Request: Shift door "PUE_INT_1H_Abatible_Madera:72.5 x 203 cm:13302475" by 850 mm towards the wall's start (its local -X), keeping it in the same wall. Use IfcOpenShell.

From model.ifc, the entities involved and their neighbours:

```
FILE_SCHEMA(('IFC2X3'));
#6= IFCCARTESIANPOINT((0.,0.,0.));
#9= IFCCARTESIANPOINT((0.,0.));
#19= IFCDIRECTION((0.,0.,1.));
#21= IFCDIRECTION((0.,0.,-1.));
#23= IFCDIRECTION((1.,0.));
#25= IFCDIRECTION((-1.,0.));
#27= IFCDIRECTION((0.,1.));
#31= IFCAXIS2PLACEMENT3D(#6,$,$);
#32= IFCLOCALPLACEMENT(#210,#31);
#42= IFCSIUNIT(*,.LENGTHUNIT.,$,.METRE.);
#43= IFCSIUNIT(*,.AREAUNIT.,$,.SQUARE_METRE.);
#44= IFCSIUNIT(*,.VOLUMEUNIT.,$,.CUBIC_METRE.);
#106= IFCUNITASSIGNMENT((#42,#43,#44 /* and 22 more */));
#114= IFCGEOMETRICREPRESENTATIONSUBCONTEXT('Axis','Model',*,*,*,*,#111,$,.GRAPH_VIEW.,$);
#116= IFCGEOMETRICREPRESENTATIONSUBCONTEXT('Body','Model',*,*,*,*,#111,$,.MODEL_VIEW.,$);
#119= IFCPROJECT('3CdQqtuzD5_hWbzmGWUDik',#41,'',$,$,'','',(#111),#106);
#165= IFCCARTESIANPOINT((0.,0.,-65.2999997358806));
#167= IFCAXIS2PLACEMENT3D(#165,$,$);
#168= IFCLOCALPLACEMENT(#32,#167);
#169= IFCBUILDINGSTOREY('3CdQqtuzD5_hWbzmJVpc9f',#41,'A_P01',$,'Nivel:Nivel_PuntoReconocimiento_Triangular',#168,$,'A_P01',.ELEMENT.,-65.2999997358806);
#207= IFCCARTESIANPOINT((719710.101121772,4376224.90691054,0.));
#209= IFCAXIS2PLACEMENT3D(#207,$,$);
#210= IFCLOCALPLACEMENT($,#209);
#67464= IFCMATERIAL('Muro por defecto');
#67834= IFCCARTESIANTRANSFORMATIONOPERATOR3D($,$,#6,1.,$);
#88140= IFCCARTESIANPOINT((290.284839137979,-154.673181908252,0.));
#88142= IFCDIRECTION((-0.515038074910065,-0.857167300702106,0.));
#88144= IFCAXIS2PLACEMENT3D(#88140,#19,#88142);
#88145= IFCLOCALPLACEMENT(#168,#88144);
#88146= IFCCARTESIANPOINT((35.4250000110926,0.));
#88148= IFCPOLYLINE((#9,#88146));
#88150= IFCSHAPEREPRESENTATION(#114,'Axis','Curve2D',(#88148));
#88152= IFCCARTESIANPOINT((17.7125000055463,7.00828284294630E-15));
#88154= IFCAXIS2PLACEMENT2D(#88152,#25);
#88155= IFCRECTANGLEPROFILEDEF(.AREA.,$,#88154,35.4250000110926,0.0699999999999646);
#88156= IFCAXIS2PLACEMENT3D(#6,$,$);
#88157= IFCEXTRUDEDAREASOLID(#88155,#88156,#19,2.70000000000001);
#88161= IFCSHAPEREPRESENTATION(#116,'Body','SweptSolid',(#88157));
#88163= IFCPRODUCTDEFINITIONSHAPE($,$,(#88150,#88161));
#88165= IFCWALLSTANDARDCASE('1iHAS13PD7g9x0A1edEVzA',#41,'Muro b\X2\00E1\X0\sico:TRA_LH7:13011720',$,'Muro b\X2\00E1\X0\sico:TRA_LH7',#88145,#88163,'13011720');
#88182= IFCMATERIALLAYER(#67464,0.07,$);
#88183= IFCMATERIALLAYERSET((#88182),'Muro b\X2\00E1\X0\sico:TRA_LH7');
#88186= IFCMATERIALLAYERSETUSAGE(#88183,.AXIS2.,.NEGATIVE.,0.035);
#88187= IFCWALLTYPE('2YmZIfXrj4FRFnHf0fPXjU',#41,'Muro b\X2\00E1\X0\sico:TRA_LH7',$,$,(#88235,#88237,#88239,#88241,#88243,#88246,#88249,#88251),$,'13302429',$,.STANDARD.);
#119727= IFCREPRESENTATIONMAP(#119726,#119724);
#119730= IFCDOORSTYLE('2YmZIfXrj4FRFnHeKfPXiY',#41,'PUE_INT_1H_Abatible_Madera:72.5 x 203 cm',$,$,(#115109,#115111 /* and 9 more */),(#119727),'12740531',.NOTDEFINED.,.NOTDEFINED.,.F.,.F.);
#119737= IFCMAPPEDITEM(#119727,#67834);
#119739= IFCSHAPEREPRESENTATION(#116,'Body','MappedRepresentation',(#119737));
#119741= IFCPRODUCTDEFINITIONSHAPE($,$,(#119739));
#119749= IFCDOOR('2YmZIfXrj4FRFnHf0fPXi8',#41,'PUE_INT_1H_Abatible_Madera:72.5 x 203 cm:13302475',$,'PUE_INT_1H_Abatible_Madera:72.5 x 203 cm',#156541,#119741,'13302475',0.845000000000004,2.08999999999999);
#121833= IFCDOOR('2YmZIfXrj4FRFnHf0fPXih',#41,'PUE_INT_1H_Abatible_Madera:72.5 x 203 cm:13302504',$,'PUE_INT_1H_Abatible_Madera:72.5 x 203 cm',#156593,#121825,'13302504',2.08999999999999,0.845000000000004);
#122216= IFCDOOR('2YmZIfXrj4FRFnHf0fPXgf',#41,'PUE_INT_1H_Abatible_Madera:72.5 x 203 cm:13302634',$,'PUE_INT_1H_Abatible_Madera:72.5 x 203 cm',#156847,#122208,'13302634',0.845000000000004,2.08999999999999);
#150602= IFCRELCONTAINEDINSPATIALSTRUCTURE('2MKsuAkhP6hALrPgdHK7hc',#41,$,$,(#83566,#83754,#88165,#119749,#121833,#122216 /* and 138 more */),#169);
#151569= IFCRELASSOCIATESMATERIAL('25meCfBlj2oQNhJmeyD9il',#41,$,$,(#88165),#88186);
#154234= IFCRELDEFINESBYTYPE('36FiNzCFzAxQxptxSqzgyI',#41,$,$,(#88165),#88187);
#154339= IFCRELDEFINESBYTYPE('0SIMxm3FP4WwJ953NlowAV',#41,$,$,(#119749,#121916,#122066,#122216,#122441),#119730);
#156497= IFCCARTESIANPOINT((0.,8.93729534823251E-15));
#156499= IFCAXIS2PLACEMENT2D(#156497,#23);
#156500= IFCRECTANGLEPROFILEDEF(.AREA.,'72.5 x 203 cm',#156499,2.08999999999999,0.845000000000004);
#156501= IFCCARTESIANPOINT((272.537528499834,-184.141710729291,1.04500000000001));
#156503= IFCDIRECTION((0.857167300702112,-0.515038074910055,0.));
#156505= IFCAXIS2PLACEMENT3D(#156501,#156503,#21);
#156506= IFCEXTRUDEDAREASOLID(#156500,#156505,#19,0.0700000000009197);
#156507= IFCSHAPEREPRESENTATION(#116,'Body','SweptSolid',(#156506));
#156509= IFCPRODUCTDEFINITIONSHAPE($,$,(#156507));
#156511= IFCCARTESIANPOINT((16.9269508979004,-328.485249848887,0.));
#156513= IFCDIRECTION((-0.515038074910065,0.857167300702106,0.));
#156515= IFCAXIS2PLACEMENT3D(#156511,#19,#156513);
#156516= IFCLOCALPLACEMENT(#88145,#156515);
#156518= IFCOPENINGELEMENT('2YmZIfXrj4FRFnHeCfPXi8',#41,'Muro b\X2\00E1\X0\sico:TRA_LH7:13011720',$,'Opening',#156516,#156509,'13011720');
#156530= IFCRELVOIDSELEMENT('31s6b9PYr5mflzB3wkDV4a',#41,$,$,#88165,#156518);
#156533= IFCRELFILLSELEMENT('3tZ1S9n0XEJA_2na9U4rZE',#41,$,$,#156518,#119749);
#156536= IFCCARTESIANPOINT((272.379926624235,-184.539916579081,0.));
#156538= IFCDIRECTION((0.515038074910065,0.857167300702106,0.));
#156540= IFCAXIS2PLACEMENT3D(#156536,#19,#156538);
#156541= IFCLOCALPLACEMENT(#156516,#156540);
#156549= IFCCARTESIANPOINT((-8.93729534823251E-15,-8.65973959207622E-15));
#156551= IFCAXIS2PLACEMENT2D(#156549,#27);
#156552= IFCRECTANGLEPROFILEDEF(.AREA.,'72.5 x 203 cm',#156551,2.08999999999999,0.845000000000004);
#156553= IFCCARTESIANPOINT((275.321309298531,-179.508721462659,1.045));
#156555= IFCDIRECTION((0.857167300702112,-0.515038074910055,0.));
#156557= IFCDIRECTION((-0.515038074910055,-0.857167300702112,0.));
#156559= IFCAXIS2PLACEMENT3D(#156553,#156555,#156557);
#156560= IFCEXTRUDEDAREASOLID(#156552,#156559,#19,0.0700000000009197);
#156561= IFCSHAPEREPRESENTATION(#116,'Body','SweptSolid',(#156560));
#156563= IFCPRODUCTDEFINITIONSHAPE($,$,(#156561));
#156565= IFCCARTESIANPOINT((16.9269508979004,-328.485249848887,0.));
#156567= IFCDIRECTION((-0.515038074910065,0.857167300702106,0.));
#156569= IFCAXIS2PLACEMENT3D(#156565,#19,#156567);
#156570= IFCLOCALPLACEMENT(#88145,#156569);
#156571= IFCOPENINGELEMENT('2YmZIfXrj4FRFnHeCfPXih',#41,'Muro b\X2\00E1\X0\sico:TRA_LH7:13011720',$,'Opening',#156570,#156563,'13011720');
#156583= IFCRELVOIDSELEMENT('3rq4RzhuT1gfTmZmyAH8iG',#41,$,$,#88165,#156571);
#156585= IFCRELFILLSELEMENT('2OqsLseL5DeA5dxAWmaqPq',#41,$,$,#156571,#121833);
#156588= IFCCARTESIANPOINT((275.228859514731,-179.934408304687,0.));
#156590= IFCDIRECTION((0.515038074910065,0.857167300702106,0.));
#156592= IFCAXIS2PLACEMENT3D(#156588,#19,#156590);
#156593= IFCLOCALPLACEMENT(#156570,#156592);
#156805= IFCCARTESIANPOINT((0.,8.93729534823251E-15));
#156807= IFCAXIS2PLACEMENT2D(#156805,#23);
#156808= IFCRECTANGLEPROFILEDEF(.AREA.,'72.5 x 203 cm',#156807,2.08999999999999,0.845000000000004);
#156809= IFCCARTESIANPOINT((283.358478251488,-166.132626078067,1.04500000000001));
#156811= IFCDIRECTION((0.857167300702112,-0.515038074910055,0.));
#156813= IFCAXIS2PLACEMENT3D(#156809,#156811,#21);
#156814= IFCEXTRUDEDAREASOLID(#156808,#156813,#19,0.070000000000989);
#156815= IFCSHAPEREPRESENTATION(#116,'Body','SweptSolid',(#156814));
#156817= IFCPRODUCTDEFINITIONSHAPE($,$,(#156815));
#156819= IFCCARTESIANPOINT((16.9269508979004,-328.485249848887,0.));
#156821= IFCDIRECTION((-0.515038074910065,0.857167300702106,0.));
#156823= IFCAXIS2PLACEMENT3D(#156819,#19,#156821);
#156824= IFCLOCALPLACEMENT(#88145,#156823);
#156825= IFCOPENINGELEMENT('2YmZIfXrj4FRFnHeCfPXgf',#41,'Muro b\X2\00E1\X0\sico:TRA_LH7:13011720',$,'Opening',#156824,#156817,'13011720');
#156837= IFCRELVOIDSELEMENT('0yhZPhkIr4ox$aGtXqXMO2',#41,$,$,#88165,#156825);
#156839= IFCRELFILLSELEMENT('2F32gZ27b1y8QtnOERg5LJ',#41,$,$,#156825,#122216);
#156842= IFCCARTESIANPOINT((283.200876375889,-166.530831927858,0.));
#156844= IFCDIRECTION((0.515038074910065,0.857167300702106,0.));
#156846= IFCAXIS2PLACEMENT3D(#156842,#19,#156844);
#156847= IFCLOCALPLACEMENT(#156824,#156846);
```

```python
import ifcopenshell
import ifcopenshell.api.geometry
import ifcopenshell.util.placement
import ifcopenshell.util.unit

model = ifcopenshell.open("model.ifc")
unit_scale = ifcopenshell.util.unit.calculate_unit_scale(model)

door = model.by_guid("2YmZIfXrj4FRFnHf0fPXi8")
opening = door.FillsVoids[0].RelatingOpeningElement
wall = opening.VoidsElements[0].RelatingBuildingElement

wall_matrix = ifcopenshell.util.placement.get_local_placement(wall.ObjectPlacement)
shift = wall_matrix[:3, 0] * -0.85 / unit_scale
before = ifcopenshell.util.placement.get_local_placement(door.ObjectPlacement)[:3, 3].copy()

# The door is placed relative to its opening, so it follows when the opening moves.
matrix = ifcopenshell.util.placement.get_local_placement(opening.ObjectPlacement)
matrix[:3, 3] += shift
ifcopenshell.api.geometry.edit_object_placement(
    model, product=opening, matrix=matrix, is_si=False, should_transform_children=True
)

after = ifcopenshell.util.placement.get_local_placement(door.ObjectPlacement)[:3, 3]
print("door moved by", (after - before).round(3) + 0.0)

model.write("model_rev.ifc")
```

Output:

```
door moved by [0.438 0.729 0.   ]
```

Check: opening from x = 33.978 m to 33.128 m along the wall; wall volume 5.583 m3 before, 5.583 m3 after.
